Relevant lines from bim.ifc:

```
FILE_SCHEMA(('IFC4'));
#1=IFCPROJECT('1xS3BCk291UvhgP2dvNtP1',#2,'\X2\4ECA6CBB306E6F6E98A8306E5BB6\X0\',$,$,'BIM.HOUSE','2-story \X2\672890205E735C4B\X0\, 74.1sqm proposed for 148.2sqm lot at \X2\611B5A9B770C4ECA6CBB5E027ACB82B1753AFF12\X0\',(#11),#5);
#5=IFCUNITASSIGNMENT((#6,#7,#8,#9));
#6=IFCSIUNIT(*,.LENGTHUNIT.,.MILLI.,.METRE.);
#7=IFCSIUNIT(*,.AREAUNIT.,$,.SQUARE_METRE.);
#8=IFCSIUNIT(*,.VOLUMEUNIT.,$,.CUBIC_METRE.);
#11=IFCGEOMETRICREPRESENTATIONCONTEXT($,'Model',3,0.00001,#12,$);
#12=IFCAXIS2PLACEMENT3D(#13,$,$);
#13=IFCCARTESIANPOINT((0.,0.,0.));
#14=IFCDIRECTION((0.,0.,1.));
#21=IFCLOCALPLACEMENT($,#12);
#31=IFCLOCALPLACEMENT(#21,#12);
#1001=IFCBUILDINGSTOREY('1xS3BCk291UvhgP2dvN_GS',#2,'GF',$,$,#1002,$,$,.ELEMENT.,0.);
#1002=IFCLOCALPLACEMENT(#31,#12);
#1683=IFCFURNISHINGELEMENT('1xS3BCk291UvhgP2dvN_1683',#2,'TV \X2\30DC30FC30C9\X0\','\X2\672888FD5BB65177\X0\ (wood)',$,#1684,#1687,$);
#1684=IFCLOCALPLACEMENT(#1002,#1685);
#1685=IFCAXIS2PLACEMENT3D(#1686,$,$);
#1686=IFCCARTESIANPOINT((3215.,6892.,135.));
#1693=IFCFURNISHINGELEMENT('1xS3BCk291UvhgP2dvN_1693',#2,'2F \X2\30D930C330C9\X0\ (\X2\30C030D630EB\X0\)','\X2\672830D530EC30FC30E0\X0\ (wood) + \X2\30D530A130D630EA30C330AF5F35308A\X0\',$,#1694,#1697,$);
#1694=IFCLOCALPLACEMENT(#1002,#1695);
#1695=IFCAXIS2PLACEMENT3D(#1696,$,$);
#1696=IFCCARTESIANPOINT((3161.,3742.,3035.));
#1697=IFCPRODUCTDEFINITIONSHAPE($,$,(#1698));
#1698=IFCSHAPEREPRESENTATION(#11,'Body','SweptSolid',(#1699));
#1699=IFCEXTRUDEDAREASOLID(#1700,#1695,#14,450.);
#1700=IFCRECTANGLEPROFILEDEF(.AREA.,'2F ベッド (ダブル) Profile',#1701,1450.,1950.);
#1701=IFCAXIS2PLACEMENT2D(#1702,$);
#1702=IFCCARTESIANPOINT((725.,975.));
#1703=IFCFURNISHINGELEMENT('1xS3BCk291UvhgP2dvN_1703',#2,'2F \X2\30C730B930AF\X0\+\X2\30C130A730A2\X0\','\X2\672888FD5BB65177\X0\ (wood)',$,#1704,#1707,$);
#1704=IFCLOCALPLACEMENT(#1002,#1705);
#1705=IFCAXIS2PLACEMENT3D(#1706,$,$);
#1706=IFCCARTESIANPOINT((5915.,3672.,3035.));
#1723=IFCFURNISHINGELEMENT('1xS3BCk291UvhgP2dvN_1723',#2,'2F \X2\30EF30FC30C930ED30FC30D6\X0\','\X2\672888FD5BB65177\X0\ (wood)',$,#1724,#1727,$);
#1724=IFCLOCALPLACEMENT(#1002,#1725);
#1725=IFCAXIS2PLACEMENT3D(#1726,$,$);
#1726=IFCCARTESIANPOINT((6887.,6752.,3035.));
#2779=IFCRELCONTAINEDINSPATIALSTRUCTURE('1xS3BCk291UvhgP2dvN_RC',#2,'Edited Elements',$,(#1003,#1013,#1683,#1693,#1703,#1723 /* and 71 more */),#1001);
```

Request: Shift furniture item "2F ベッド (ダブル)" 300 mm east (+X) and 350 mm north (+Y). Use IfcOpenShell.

```python
import ifcopenshell
import ifcopenshell.api.geometry
import ifcopenshell.util.placement
import ifcopenshell.util.unit

model = ifcopenshell.open("bim.ifc")
unit_scale = ifcopenshell.util.unit.calculate_unit_scale(model)

item = model.by_guid("1xS3BCk291UvhgP2dvN_1693")
matrix = ifcopenshell.util.placement.get_local_placement(item.ObjectPlacement)
matrix[0, 3] += 0.3 / unit_scale
matrix[1, 3] += 0.35 / unit_scale
ifcopenshell.api.geometry.edit_object_placement(model, product=item, matrix=matrix, is_si=False)

print(ifcopenshell.util.placement.get_local_placement(item.ObjectPlacement).round(3) + 0.0)

model.write("bim_updated.ifc")
```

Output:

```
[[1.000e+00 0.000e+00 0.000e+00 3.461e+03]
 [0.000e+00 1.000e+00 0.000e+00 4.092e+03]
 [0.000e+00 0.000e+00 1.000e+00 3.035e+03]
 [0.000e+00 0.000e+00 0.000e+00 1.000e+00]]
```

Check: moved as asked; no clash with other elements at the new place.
